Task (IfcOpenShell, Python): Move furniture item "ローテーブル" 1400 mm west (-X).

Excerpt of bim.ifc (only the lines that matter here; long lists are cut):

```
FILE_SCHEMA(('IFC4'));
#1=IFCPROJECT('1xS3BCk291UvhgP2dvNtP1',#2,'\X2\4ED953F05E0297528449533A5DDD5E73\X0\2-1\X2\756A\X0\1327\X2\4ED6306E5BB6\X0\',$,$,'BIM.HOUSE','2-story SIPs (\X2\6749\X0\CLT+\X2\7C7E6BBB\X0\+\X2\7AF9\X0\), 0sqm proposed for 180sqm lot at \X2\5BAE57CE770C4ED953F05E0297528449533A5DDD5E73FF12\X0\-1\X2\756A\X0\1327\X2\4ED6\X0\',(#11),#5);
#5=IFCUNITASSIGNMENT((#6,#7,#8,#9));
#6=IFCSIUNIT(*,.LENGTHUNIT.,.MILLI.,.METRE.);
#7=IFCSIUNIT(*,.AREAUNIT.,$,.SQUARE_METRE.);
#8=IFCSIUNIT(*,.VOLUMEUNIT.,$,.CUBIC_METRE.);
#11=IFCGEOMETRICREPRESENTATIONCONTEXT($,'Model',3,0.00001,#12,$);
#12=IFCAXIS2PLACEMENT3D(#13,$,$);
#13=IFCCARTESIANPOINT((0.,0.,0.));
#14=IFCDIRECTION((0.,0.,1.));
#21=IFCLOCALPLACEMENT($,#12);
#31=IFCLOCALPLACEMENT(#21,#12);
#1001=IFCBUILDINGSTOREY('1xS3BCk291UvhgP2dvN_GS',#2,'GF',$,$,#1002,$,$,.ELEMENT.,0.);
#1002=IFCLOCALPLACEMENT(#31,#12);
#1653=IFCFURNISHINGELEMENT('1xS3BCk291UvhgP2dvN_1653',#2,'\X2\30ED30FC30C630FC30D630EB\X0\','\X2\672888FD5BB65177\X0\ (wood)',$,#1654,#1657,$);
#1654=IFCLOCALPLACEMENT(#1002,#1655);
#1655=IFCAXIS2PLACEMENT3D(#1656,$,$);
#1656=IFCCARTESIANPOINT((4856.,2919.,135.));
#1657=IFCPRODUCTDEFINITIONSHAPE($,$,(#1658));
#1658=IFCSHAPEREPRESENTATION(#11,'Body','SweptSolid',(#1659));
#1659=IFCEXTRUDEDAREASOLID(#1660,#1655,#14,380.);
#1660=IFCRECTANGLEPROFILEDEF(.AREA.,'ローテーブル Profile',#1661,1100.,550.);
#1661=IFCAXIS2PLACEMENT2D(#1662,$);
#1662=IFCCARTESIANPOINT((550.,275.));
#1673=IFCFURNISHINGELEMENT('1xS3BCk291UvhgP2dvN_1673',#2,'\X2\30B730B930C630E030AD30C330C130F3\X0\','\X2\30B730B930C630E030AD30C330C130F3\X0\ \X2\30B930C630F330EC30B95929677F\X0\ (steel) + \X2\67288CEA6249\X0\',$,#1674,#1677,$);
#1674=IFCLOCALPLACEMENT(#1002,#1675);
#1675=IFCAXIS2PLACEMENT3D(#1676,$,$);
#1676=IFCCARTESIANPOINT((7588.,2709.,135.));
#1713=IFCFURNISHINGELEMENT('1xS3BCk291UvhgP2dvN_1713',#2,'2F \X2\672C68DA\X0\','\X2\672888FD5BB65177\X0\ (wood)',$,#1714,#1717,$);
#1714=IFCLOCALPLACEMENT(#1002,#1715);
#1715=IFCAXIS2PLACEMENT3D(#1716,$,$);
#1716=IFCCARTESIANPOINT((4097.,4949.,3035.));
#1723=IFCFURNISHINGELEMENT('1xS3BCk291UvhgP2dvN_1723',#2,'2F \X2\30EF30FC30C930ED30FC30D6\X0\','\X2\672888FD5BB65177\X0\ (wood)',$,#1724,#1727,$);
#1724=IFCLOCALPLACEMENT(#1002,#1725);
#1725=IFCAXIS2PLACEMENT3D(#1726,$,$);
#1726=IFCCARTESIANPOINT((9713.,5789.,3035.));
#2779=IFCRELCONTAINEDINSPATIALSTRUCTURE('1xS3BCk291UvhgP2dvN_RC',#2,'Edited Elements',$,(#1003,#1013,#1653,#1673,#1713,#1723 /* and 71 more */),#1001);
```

```python
import ifcopenshell
import ifcopenshell.api.geometry
import ifcopenshell.util.placement
import ifcopenshell.util.unit

model = ifcopenshell.open("bim.ifc")
unit_scale = ifcopenshell.util.unit.calculate_unit_scale(model)

item = model.by_id(1653)
matrix = ifcopenshell.util.placement.get_local_placement(item.ObjectPlacement)
matrix[0, 3] -= 1.4 / unit_scale
ifcopenshell.api.geometry.edit_object_placement(model, product=item, matrix=matrix, is_si=False)

print(ifcopenshell.util.placement.get_local_placement(item.ObjectPlacement).round(3) + 0.0)

model.write("bim-out.ifc")
```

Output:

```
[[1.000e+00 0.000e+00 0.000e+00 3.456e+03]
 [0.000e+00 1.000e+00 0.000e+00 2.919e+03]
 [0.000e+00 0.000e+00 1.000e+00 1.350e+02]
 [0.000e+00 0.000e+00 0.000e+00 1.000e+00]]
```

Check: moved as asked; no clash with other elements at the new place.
